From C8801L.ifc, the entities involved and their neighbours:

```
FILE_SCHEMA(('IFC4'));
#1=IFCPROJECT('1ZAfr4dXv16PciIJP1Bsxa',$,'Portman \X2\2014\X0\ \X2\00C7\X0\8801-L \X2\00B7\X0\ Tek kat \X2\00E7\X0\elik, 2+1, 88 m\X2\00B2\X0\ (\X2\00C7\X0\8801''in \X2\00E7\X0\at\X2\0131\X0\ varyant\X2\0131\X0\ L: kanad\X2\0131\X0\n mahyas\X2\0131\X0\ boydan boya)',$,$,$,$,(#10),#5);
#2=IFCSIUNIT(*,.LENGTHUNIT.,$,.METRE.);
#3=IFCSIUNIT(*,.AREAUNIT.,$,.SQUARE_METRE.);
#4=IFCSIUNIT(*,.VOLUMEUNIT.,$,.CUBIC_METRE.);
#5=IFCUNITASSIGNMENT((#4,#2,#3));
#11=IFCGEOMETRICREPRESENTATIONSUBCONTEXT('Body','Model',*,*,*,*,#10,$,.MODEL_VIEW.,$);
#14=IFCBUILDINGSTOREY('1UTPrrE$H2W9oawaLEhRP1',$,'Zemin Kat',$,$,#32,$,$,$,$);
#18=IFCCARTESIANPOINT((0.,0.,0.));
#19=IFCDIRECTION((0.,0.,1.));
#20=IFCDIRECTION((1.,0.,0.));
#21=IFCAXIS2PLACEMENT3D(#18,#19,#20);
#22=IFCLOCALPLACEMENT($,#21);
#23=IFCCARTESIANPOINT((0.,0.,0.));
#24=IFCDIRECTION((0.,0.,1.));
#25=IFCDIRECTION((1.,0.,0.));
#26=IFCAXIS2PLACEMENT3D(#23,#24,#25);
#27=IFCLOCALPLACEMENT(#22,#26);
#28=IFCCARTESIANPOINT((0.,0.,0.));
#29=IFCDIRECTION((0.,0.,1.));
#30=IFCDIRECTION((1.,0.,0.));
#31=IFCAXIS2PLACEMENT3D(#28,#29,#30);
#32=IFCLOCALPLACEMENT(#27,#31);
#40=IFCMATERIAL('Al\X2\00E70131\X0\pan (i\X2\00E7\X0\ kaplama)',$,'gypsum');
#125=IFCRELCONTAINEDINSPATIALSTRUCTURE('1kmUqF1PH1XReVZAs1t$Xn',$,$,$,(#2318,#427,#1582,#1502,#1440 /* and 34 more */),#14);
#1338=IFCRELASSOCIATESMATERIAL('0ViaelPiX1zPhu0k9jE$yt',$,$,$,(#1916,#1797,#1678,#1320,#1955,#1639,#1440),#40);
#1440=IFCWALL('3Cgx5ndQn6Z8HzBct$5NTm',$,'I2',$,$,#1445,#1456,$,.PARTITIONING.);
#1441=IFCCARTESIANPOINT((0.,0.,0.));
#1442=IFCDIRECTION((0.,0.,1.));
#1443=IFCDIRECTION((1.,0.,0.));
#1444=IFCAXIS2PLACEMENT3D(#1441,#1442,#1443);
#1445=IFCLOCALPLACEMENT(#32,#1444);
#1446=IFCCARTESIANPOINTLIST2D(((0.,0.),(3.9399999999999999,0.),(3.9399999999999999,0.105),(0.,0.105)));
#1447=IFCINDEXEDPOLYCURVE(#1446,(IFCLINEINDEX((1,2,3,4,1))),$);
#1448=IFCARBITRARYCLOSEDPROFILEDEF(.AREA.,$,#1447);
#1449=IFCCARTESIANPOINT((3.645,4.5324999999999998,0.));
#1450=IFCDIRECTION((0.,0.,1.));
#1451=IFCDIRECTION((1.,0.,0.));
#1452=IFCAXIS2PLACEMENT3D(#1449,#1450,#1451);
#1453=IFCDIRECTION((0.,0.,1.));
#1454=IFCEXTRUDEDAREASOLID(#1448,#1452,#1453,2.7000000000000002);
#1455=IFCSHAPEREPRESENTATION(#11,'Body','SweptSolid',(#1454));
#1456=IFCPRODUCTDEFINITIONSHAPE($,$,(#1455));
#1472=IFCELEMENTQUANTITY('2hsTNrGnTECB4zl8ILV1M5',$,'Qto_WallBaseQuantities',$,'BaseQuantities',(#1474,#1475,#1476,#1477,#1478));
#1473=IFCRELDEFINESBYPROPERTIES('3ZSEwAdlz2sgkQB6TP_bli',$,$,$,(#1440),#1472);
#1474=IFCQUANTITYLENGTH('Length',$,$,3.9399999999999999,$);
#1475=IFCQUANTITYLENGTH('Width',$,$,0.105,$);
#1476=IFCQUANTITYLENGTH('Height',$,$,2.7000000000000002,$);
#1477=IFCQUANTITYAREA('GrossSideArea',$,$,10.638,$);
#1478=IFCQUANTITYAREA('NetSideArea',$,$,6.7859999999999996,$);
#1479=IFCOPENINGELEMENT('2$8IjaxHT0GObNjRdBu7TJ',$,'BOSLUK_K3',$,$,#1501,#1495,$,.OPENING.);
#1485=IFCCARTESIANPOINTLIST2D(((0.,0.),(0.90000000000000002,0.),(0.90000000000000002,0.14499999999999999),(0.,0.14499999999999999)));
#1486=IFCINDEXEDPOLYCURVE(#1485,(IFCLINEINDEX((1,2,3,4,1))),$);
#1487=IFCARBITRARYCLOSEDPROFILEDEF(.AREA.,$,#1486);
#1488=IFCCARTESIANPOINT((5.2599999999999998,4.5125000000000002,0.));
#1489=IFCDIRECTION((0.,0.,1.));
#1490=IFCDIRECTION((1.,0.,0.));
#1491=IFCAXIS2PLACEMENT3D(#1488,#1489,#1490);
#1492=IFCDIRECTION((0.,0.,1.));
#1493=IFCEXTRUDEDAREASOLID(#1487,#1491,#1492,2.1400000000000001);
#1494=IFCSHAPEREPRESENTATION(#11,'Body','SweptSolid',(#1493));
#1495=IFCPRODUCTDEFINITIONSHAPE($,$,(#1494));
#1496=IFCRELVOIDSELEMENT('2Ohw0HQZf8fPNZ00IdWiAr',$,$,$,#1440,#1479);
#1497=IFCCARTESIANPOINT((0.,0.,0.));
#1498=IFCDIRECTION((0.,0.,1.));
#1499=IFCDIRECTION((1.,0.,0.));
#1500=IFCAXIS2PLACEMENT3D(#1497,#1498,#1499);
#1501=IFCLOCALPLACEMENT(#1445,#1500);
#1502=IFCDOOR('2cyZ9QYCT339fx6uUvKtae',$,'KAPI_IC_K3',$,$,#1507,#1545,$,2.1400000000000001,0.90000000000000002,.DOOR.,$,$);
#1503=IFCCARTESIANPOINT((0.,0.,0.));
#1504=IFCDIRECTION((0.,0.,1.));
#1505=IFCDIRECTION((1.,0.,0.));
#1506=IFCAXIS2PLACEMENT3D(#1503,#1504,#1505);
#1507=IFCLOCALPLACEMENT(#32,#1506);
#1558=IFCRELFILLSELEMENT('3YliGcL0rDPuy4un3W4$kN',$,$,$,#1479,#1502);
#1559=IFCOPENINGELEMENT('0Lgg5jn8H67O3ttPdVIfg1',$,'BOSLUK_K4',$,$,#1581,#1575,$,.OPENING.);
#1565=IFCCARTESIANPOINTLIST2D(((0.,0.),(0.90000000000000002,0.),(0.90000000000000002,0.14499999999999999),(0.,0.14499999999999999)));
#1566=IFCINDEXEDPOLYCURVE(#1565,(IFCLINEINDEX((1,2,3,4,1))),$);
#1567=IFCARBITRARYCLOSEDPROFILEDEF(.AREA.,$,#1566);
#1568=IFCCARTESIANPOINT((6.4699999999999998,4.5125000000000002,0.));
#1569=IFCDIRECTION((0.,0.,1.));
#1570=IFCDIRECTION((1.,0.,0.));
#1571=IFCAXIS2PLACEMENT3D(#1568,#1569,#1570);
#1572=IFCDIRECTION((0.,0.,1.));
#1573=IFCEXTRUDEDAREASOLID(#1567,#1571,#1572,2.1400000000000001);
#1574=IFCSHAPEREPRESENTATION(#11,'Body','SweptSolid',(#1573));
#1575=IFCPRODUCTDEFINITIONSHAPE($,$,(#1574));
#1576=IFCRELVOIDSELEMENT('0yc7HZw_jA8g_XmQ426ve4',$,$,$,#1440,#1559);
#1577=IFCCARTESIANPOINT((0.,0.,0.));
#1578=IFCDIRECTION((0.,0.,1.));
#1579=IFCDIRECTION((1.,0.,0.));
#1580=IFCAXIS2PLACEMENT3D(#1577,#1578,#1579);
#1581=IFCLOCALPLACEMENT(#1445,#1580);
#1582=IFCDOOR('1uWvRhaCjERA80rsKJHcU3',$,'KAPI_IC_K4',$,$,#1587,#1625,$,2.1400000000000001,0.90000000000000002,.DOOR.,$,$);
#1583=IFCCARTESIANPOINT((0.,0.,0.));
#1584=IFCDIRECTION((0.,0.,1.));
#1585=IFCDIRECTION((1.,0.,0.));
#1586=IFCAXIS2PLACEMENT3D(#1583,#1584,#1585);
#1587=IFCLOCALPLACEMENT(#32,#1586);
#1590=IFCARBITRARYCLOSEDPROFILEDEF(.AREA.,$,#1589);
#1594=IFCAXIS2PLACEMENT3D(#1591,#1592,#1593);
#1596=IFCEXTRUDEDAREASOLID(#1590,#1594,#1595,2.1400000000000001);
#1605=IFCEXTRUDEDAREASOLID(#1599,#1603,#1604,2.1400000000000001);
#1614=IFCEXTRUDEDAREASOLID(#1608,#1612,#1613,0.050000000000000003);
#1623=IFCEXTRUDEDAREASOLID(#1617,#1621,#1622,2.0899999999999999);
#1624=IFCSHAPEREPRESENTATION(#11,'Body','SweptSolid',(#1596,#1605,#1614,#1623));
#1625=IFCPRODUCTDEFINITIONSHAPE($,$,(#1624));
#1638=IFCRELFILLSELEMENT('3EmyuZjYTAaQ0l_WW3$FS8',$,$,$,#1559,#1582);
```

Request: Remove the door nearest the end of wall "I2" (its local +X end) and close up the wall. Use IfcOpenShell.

```python
import ifcopenshell
import ifcopenshell.api.feature
import ifcopenshell.api.pset
import ifcopenshell.api.root
import ifcopenshell.geom
import ifcopenshell.util.element
import ifcopenshell.util.shape
import ifcopenshell.util.unit

model = ifcopenshell.open("C8801L.ifc")
area_scale = ifcopenshell.util.unit.calculate_unit_scale(model, "AREAUNIT")
settings = ifcopenshell.geom.settings()


def volume(element):
    """Net volume in cubic metres, openings subtracted."""
    shape = ifcopenshell.geom.create_shape(settings, element)
    return ifcopenshell.util.shape.get_volume(shape.geometry)


door = model.by_guid("1uWvRhaCjERA80rsKJHcU3")
opening = door.FillsVoids[0].RelatingOpeningElement
wall = opening.VoidsElements[0].RelatingBuildingElement
before = volume(wall)

ifcopenshell.api.root.remove_product(model, product=door)
ifcopenshell.api.feature.remove_feature(model, feature=opening)

after = volume(wall)
thickness = 0.105  # wall thickness in metres

# Update the wall's stored quantities.
qto = model.by_id(ifcopenshell.util.element.get_pset(wall, "Qto_WallBaseQuantities", should_inherit=False)["id"])
ifcopenshell.api.pset.edit_qto(model, qto=qto, properties={"NetSideArea": after / thickness / area_scale})

print(f"wall volume {before:.3f} -> {after:.3f} m3")

model.write("C8801L_updated.ifc")
```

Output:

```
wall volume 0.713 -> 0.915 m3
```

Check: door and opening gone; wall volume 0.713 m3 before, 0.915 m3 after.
